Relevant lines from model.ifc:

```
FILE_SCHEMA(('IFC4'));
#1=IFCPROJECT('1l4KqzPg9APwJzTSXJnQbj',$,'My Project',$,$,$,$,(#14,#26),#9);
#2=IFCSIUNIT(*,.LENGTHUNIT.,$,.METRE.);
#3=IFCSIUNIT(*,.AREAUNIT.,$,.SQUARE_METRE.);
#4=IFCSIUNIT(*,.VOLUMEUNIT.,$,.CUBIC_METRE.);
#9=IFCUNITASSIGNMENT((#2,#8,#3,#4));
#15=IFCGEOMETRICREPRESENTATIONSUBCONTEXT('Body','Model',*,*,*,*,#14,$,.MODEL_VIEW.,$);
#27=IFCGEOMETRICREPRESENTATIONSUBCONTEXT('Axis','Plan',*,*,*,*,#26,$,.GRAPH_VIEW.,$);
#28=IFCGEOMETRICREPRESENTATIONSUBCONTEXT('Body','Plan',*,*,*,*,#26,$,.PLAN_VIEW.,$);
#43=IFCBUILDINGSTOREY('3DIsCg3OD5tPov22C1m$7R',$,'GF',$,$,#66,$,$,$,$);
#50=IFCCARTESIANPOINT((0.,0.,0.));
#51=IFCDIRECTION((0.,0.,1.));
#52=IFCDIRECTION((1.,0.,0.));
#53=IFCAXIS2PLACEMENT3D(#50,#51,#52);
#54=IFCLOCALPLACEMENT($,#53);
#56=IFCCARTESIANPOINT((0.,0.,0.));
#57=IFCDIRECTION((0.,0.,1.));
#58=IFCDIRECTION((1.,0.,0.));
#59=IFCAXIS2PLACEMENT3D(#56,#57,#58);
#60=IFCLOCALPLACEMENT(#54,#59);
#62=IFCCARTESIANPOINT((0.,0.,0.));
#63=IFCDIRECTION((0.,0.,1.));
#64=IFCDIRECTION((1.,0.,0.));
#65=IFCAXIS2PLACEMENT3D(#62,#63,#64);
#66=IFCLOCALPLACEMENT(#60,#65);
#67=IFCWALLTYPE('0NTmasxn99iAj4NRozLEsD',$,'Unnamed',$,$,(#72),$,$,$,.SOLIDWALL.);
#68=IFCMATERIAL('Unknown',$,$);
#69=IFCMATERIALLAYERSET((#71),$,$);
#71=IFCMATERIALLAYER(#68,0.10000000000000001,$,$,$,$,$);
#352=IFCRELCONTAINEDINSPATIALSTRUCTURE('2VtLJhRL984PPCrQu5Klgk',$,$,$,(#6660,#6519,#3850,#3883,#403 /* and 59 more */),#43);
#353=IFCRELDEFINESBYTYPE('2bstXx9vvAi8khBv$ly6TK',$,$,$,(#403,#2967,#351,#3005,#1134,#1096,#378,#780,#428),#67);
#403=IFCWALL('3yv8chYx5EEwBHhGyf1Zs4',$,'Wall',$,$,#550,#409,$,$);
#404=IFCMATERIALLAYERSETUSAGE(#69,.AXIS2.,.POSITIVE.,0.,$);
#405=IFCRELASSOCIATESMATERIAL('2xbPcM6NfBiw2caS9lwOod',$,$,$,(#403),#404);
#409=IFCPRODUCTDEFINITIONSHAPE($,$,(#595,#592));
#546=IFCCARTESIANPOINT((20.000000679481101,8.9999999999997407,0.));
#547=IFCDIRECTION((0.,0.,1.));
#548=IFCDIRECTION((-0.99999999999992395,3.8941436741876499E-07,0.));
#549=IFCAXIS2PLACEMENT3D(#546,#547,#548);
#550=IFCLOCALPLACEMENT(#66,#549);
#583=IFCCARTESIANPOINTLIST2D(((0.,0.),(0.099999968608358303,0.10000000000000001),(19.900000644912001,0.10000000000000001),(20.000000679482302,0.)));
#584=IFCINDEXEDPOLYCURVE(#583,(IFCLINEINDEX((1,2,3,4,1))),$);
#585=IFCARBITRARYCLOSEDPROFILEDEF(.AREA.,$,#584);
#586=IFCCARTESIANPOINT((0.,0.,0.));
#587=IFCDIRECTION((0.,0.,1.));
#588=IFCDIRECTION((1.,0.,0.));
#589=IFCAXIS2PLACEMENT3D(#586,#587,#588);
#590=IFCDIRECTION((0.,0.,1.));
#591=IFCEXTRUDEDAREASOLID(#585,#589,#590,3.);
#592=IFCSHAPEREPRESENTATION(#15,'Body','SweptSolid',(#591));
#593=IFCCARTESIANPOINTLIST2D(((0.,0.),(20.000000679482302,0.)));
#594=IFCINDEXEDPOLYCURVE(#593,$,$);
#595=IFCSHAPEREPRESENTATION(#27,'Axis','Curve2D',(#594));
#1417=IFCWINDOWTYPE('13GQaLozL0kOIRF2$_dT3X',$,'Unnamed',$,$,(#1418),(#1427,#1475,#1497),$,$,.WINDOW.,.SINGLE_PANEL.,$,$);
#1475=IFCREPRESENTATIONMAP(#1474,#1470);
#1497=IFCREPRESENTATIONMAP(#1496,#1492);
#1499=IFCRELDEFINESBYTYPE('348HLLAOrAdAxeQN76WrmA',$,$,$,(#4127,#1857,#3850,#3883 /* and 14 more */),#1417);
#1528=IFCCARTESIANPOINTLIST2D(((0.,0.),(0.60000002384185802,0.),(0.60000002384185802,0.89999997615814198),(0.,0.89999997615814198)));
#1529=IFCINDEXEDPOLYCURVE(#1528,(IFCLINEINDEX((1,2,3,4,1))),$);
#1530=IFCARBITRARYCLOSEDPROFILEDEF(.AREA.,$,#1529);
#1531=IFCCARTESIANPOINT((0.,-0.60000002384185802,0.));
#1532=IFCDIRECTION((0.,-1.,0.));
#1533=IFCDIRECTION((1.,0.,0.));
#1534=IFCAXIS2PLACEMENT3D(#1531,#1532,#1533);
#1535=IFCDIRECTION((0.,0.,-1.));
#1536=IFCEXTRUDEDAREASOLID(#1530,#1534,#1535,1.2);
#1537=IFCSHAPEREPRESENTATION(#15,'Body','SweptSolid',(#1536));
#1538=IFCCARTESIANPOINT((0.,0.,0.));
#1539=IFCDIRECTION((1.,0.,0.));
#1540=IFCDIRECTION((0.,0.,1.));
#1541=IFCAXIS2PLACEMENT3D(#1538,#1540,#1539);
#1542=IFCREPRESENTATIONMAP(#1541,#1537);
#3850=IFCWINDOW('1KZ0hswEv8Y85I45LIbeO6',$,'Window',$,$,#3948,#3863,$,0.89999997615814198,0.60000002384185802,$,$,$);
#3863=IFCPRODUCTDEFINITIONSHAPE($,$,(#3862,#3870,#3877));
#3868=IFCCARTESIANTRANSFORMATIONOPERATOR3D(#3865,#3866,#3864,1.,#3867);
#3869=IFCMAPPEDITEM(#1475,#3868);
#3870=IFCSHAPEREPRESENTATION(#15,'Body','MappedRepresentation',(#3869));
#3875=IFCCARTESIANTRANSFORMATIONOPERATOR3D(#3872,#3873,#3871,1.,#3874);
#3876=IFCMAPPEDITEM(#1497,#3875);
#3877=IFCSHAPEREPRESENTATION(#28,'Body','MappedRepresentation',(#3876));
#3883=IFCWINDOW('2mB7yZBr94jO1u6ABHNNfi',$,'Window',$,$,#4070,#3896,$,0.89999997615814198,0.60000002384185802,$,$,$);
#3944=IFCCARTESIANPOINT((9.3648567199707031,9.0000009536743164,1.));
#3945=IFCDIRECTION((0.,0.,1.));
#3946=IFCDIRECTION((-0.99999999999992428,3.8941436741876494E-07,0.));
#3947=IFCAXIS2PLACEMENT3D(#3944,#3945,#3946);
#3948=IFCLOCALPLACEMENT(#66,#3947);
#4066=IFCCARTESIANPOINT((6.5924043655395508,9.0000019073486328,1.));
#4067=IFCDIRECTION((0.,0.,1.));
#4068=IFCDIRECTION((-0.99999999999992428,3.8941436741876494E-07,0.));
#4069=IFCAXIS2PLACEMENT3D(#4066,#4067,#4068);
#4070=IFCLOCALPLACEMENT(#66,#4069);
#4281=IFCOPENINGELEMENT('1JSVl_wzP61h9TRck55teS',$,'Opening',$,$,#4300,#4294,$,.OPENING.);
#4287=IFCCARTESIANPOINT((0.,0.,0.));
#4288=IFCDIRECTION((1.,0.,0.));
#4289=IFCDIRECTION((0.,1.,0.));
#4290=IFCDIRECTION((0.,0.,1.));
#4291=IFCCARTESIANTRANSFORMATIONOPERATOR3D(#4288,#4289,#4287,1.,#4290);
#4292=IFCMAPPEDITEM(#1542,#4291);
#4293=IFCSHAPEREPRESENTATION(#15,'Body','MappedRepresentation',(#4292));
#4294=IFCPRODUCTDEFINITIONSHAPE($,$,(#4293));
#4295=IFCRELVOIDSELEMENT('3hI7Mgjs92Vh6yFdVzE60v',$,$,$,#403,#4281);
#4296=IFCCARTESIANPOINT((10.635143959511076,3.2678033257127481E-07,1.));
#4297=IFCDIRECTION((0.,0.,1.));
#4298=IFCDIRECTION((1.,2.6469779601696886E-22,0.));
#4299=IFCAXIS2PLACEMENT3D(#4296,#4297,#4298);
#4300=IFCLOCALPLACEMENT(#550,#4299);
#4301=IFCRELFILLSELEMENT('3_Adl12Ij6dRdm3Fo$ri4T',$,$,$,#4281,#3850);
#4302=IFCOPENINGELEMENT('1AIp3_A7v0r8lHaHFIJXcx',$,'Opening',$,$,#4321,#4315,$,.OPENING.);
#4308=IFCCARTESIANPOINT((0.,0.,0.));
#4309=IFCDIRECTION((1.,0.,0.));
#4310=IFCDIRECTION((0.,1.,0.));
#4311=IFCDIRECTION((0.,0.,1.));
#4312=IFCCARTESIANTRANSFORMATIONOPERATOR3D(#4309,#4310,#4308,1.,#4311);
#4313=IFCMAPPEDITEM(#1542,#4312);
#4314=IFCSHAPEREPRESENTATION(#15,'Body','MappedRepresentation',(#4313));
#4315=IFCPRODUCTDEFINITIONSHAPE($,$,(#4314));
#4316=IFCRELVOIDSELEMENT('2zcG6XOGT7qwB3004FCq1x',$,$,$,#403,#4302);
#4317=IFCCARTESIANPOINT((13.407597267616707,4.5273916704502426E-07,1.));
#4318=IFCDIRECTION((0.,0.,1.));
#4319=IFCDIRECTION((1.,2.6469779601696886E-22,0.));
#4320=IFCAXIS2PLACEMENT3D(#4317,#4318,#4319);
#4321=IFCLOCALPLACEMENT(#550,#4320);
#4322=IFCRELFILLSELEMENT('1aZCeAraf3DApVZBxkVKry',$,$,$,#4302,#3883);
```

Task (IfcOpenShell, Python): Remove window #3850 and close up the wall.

```python
import ifcopenshell
import ifcopenshell.api.feature
import ifcopenshell.api.root
import ifcopenshell.geom
import ifcopenshell.util.shape

model = ifcopenshell.open("model.ifc")
settings = ifcopenshell.geom.settings()


def volume(element):
    """Net volume in cubic metres, openings subtracted."""
    shape = ifcopenshell.geom.create_shape(settings, element)
    return ifcopenshell.util.shape.get_volume(shape.geometry)


window = model.by_guid("1KZ0hswEv8Y85I45LIbeO6")
opening = window.FillsVoids[0].RelatingOpeningElement
wall = opening.VoidsElements[0].RelatingBuildingElement
before = volume(wall)

ifcopenshell.api.root.remove_product(model, product=window)
ifcopenshell.api.feature.remove_feature(model, feature=opening)

after = volume(wall)

print(f"wall volume {before:.3f} -> {after:.3f} m3")

model.write("model-out.ifc")
```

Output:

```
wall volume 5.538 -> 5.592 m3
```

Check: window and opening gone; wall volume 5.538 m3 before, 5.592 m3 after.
